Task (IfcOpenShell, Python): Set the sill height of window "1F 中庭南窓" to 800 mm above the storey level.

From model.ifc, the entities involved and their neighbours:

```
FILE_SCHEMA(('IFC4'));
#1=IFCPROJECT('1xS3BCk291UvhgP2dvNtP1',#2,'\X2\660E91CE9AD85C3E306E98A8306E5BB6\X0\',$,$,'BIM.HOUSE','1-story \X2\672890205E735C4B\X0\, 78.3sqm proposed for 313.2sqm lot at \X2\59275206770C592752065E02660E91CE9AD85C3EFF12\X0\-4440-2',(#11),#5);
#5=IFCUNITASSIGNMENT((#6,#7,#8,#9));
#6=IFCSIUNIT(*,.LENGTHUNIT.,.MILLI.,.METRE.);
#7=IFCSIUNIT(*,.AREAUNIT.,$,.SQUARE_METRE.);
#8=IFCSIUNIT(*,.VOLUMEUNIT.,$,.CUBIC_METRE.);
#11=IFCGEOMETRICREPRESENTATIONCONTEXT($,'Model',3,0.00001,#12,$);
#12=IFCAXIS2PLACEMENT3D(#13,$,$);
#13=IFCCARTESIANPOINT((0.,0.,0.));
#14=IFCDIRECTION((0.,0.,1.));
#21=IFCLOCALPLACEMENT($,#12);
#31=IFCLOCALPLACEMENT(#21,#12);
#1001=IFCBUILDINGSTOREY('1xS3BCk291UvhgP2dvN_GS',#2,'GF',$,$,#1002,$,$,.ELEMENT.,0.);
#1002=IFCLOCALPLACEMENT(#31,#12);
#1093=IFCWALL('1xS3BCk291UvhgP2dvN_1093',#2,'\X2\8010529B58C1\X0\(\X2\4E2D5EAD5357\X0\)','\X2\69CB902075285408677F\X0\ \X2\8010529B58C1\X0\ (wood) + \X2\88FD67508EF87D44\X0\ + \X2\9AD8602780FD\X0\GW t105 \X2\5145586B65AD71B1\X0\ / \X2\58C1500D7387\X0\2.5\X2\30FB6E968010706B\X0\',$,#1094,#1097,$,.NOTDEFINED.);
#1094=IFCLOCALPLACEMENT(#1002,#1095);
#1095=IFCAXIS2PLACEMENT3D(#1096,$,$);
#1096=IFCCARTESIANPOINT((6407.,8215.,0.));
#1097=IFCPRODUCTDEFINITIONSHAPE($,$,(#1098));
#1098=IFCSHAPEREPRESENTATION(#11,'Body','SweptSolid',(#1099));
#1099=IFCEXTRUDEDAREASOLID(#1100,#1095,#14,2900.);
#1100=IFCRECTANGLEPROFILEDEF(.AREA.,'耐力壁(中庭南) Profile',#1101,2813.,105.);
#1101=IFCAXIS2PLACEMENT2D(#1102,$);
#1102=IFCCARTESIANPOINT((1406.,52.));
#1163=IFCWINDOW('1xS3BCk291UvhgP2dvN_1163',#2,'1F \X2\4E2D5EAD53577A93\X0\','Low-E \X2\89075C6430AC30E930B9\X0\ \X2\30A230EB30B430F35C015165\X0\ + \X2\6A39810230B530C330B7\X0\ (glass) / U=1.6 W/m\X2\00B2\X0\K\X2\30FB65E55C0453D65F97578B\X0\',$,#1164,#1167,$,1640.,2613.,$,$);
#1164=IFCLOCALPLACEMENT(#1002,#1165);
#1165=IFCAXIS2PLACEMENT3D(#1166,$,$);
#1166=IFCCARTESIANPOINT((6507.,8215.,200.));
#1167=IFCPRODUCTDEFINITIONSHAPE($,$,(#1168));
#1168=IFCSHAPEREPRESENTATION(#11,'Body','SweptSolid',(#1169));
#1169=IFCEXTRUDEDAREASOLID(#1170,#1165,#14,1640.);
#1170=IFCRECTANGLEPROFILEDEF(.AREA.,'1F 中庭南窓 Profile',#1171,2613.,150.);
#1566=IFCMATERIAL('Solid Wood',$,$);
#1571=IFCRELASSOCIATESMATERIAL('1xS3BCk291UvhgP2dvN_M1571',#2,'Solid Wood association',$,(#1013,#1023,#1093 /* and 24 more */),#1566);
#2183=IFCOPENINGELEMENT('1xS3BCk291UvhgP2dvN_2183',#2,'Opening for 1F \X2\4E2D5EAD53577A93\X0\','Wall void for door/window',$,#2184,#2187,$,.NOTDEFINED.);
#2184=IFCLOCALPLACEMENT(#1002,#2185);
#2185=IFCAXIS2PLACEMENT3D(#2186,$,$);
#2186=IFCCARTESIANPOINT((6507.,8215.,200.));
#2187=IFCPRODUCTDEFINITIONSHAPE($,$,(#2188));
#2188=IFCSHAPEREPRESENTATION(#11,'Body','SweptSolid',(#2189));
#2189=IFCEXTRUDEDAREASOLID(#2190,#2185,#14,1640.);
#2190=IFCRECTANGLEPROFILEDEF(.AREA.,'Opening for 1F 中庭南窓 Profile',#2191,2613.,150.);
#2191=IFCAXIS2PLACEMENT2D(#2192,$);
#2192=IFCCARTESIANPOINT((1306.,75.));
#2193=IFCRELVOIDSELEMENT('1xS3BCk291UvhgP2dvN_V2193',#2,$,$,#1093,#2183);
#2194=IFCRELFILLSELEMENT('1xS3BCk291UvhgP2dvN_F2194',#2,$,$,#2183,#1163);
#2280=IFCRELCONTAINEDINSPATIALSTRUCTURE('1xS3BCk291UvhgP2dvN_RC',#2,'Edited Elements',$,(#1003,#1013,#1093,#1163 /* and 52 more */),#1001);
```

```python
import numpy as np
import ifcopenshell
import ifcopenshell.api.geometry
import ifcopenshell.geom
import ifcopenshell.util.element
import ifcopenshell.util.placement
import ifcopenshell.util.shape
import ifcopenshell.util.unit

model = ifcopenshell.open("model.ifc")
unit_scale = ifcopenshell.util.unit.calculate_unit_scale(model)

window = model.by_guid("1xS3BCk291UvhgP2dvN_1163")
opening = window.FillsVoids[0].RelatingOpeningElement
storey = ifcopenshell.util.element.get_container(window, ifc_class="IfcBuildingStorey")
level = ifcopenshell.util.placement.get_local_placement(storey.ObjectPlacement)[2, 3]

# The opening's origin need not be at the sill, so measure its lowest point.
shape = ifcopenshell.geom.create_shape(ifcopenshell.geom.settings(), opening)
bottom = ifcopenshell.util.shape.get_shape_bottom_elevation(shape, shape.geometry) / unit_scale
dz = level + 0.8 / unit_scale - bottom

shift = np.array([0.0, 0.0, dz])
# The window is not placed relative to its opening, so move both.
for product in (opening, window):
    matrix = ifcopenshell.util.placement.get_local_placement(product.ObjectPlacement)
    matrix[:3, 3] += shift
    ifcopenshell.api.geometry.edit_object_placement(model, product=product, matrix=matrix, is_si=False)

print(f"moved by {dz * unit_scale:+.3f} m")

model.write("model_rev.ifc")
```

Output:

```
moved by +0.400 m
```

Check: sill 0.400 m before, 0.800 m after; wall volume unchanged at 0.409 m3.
